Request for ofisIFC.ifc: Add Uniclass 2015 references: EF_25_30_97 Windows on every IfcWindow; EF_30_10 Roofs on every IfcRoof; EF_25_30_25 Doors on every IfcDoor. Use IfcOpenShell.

First a look at what the model holds.

```python
import ifcopenshell

model = ifcopenshell.open("ofisIFC.ifc")
print(model.schema)
print("classifications:", [c.Name for c in model.by_type("IfcClassification")])
for ifc_class in ("IfcDoor", "IfcRoof", "IfcStair", "IfcWall", "IfcWindow"):
    print(ifc_class, len(model.by_type(ifc_class)))
```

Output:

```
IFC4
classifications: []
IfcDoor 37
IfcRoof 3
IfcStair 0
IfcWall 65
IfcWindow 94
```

```python
import ifcopenshell
import ifcopenshell.api.classification

model = ifcopenshell.open("ofisIFC.ifc")

system = ifcopenshell.api.classification.add_classification(model, classification="Uniclass 2015")

codes = {
    "IfcWindow": ("EF_25_30_97", "Windows"),
    "IfcRoof": ("EF_30_10", "Roofs"),
    "IfcDoor": ("EF_25_30_25", "Doors"),
}
for ifc_class, (code, name) in codes.items():
    products = model.by_type(ifc_class)
    ifcopenshell.api.classification.add_reference(
        model, products=products, classification=system, identification=code, name=name
    )
    print(code, len(products))

model.write("ofisIFC_v2.ifc")
```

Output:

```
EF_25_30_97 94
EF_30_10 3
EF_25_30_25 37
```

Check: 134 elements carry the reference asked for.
